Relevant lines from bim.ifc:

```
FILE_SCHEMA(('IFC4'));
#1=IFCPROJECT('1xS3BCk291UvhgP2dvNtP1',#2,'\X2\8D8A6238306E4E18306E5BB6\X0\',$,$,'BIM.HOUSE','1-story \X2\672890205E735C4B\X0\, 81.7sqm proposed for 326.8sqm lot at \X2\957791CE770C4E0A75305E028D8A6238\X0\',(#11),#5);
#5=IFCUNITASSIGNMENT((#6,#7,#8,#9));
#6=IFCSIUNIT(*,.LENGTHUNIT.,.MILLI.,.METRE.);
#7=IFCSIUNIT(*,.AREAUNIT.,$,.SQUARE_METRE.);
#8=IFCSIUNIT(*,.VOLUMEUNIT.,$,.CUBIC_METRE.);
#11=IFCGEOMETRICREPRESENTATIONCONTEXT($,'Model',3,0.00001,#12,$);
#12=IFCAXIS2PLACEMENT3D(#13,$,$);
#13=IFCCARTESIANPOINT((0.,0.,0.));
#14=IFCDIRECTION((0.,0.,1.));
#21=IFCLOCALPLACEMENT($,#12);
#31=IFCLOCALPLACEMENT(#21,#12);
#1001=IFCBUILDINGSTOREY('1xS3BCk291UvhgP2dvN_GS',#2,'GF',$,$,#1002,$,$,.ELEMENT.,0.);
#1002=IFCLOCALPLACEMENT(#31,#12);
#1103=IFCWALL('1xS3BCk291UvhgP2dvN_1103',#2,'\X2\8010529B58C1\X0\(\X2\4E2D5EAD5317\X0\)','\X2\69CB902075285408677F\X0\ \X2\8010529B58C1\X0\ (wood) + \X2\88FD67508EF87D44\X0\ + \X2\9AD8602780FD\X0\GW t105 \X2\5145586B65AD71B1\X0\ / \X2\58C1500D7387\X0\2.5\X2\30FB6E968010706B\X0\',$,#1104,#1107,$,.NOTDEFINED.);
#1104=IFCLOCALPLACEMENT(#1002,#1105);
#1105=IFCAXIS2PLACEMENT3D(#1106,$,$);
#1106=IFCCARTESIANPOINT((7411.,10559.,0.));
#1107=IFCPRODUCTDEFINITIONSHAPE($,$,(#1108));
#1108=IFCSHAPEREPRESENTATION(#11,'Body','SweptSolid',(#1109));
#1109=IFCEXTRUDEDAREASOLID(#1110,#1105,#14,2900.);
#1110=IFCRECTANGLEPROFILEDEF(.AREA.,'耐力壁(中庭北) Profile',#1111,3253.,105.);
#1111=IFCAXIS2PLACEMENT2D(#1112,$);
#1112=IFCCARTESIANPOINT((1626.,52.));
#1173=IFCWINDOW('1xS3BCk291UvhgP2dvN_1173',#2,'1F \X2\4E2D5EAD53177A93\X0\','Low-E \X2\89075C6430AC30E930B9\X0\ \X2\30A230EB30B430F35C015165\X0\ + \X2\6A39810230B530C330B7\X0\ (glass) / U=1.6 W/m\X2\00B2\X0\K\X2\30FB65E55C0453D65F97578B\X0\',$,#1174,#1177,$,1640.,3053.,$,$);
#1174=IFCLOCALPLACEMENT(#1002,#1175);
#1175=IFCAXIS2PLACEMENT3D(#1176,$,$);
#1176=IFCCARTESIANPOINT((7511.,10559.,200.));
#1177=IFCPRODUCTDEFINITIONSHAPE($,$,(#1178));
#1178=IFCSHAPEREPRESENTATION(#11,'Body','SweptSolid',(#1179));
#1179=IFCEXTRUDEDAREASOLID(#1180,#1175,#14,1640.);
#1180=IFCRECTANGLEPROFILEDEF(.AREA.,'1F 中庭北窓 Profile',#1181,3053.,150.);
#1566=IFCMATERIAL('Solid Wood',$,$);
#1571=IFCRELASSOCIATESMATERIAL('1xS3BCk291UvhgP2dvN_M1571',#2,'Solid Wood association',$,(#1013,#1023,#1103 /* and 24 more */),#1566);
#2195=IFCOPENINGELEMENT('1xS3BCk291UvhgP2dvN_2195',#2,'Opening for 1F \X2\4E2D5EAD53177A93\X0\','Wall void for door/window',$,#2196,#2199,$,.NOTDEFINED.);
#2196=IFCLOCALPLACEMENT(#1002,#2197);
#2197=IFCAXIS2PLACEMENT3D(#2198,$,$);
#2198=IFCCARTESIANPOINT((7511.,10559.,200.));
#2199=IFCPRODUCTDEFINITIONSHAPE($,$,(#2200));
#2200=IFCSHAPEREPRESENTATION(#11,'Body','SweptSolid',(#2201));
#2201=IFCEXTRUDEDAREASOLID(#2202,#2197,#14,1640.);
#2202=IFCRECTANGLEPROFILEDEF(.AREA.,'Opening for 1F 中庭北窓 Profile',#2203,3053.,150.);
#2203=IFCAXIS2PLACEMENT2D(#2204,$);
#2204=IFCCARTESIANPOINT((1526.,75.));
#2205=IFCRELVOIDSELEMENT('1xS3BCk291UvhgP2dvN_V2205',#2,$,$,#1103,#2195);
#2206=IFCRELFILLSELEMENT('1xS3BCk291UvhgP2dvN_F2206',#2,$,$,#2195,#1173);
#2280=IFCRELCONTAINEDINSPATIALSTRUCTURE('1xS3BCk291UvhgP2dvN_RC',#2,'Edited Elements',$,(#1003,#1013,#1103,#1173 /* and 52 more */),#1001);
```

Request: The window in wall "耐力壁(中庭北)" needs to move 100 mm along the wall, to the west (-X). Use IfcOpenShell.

```python
import ifcopenshell
import ifcopenshell.api.geometry
import ifcopenshell.util.placement
import ifcopenshell.util.unit

model = ifcopenshell.open("bim.ifc")
unit_scale = ifcopenshell.util.unit.calculate_unit_scale(model)

window = model.by_id(1173)
opening = window.FillsVoids[0].RelatingOpeningElement
wall = opening.VoidsElements[0].RelatingBuildingElement

wall_matrix = ifcopenshell.util.placement.get_local_placement(wall.ObjectPlacement)
shift = wall_matrix[:3, 0] * -0.1 / unit_scale
before = ifcopenshell.util.placement.get_local_placement(window.ObjectPlacement)[:3, 3].copy()

# The window is not placed relative to its opening, so move both.
for product in (opening, window):
    matrix = ifcopenshell.util.placement.get_local_placement(product.ObjectPlacement)
    matrix[:3, 3] += shift
    ifcopenshell.api.geometry.edit_object_placement(model, product=product, matrix=matrix, is_si=False)

after = ifcopenshell.util.placement.get_local_placement(window.ObjectPlacement)[:3, 3]
print("window moved by", (after - before).round(3) + 0.0)

model.write("bim_rev.ifc")
```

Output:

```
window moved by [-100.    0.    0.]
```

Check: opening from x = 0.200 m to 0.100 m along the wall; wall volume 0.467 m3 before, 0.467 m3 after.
